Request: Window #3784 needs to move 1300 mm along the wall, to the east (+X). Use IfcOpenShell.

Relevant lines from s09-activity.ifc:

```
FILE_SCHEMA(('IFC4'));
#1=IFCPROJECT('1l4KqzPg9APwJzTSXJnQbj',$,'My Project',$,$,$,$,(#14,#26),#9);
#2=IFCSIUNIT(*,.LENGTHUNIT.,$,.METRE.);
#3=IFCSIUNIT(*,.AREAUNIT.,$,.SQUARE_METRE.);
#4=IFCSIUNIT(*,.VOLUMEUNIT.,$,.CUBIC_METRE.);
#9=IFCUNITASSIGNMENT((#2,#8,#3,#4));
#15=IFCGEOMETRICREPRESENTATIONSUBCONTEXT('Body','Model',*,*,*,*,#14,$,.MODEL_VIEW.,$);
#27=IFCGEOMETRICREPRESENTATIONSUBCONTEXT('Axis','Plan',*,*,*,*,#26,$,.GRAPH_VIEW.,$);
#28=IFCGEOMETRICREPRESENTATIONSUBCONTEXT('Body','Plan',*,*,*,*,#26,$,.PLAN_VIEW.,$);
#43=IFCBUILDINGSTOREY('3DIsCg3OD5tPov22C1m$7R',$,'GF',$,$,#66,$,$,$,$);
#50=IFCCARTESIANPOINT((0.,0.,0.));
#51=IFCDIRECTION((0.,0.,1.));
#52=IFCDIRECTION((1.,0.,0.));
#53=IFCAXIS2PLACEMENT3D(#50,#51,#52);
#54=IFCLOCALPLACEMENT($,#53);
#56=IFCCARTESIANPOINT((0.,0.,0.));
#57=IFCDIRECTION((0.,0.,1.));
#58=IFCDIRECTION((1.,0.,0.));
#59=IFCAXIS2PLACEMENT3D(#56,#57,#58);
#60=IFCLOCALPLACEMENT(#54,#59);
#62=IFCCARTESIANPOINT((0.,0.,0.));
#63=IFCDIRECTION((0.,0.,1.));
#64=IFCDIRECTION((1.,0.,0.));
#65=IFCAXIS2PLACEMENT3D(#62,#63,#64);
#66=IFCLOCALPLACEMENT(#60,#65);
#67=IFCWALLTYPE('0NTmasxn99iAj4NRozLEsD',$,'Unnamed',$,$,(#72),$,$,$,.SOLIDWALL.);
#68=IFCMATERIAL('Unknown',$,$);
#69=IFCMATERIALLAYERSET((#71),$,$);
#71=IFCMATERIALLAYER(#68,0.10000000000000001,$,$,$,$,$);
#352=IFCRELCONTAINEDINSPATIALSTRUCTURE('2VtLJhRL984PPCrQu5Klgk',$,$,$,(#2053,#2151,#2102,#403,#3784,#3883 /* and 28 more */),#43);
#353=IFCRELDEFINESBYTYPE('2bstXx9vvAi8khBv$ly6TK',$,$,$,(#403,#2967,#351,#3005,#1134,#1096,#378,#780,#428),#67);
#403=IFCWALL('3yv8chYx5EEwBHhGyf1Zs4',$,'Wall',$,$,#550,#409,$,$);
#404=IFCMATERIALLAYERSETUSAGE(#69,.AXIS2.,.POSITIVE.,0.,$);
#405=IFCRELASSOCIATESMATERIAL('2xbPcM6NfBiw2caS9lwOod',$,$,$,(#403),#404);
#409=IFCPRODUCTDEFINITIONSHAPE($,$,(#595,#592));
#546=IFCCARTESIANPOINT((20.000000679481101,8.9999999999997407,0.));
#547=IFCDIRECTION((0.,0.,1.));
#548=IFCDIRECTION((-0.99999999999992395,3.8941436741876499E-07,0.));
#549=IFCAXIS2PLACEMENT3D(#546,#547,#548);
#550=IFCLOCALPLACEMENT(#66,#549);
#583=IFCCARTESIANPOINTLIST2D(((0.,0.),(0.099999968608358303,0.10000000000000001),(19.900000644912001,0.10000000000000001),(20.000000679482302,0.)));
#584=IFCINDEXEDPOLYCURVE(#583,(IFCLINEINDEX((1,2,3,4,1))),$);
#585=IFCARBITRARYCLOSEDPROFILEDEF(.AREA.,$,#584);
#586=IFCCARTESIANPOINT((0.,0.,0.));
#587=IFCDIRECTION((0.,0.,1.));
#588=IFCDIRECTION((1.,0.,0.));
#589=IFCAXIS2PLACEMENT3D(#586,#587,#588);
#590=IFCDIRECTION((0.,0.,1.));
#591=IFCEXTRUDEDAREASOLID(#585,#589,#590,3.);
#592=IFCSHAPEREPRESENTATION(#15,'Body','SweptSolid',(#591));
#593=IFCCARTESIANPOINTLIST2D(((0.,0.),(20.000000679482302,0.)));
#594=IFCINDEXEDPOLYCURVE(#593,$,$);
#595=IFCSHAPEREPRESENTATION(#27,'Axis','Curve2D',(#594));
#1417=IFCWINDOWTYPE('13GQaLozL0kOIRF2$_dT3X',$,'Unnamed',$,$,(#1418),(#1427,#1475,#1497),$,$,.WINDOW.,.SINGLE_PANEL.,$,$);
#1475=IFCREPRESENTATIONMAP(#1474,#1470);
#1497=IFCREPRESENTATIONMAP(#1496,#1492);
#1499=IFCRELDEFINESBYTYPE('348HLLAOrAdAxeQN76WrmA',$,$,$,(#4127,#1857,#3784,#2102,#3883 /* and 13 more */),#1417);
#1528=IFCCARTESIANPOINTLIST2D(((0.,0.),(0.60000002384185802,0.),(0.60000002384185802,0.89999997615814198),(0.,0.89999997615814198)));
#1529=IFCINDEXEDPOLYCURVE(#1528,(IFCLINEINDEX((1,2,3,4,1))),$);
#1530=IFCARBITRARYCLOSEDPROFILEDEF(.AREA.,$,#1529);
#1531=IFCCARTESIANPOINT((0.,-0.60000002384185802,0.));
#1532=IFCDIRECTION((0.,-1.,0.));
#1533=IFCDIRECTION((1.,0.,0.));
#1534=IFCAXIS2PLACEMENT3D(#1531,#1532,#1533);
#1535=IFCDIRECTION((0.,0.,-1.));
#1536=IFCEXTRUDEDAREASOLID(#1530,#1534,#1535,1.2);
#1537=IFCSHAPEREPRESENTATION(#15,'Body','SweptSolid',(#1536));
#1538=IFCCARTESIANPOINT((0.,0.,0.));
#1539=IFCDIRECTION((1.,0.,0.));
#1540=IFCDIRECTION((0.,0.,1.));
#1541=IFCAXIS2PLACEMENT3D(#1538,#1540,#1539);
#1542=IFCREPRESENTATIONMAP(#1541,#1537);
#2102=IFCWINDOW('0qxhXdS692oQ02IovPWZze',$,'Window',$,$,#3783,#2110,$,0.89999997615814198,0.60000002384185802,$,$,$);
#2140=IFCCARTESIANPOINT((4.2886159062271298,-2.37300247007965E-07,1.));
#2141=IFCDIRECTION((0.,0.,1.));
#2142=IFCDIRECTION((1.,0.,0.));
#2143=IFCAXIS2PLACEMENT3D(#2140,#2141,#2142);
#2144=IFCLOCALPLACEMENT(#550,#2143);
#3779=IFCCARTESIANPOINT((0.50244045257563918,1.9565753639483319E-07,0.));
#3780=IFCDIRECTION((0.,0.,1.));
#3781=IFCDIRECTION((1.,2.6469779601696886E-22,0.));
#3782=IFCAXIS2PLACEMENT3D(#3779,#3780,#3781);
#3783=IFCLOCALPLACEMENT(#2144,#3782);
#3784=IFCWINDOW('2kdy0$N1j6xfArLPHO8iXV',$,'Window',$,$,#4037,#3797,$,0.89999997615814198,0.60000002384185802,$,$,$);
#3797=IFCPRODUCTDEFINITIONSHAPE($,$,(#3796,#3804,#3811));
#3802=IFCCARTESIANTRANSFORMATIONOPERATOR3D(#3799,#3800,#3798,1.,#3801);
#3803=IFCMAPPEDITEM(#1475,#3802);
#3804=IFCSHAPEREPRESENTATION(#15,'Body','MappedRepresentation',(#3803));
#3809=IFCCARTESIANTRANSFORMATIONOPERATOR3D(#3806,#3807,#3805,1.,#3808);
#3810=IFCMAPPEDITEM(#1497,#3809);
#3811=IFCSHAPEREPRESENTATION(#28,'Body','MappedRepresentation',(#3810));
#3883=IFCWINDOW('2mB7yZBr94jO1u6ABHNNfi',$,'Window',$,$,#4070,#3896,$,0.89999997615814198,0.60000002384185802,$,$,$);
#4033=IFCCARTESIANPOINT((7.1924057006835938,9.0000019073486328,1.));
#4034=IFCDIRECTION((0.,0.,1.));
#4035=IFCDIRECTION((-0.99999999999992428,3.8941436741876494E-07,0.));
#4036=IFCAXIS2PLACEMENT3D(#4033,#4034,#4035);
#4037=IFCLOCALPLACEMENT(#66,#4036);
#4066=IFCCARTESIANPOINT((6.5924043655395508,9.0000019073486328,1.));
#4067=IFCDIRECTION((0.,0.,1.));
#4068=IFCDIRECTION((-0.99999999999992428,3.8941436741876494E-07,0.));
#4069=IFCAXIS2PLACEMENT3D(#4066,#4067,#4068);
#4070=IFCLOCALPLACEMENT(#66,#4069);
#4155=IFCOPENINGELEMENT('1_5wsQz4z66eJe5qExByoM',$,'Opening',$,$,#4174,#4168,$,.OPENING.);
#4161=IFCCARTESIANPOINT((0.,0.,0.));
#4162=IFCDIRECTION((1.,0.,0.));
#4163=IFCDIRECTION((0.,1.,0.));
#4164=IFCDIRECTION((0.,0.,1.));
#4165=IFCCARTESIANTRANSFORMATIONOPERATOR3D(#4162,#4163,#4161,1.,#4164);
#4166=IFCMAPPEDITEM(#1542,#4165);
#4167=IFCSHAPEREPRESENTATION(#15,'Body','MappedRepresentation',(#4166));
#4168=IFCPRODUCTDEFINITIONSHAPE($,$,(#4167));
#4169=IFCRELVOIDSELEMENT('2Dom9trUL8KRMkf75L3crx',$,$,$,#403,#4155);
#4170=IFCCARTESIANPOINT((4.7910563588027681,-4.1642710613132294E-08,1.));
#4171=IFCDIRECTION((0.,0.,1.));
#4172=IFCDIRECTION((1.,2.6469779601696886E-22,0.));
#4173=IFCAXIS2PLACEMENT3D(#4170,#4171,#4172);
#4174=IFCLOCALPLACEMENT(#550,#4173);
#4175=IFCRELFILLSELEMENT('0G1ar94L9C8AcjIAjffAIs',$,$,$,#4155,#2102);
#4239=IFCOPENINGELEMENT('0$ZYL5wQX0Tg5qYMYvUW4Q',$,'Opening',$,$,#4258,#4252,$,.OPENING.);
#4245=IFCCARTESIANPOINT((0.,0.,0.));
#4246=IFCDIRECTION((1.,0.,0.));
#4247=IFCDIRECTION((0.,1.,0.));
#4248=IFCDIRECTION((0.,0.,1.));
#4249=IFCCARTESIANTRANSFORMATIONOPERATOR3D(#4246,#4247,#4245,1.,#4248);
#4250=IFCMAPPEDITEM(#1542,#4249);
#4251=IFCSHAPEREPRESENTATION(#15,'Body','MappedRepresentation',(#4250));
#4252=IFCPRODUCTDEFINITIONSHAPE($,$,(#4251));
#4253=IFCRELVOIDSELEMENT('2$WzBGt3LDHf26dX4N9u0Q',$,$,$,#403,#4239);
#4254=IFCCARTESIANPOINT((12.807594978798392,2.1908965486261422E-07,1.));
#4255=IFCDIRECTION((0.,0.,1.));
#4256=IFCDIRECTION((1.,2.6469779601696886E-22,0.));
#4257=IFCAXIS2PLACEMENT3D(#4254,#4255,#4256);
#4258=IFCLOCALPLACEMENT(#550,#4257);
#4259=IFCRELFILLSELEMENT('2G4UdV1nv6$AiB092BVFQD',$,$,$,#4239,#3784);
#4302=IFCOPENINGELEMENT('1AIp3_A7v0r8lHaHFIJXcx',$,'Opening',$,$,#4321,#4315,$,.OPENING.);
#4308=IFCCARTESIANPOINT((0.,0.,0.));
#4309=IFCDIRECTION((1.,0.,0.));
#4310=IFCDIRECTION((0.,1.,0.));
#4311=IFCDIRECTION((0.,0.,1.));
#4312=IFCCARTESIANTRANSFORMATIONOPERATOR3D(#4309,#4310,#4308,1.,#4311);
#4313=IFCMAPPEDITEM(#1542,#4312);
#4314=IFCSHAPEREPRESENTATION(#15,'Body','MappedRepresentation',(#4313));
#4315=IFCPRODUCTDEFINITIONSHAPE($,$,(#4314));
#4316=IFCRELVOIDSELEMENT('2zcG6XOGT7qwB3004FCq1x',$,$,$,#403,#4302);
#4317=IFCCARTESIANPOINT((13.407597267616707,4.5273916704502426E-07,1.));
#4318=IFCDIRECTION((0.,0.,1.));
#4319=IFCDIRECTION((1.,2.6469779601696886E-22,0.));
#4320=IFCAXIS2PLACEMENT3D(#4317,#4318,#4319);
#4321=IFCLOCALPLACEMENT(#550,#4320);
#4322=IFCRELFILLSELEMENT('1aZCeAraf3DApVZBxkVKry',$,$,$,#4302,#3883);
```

```python
import ifcopenshell
import ifcopenshell.api.geometry
import ifcopenshell.util.placement
import ifcopenshell.util.unit

model = ifcopenshell.open("s09-activity.ifc")
unit_scale = ifcopenshell.util.unit.calculate_unit_scale(model)

window = model.by_guid("2kdy0$N1j6xfArLPHO8iXV")
opening = window.FillsVoids[0].RelatingOpeningElement
wall = opening.VoidsElements[0].RelatingBuildingElement

wall_matrix = ifcopenshell.util.placement.get_local_placement(wall.ObjectPlacement)
shift = wall_matrix[:3, 0] * -1.3 / unit_scale
before = ifcopenshell.util.placement.get_local_placement(window.ObjectPlacement)[:3, 3].copy()

# The window is not placed relative to its opening, so move both.
for product in (opening, window):
    matrix = ifcopenshell.util.placement.get_local_placement(product.ObjectPlacement)
    matrix[:3, 3] += shift
    ifcopenshell.api.geometry.edit_object_placement(model, product=product, matrix=matrix, is_si=False)

after = ifcopenshell.util.placement.get_local_placement(window.ObjectPlacement)[:3, 3]
print("window moved by", (after - before).round(3) + 0.0)

model.write("s09-activity_rev.ifc")
```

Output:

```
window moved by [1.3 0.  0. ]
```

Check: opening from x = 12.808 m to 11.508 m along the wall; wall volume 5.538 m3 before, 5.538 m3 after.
